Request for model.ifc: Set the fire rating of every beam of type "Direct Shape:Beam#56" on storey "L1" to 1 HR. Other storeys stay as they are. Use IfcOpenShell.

First a look at what the model holds.

```python
import ifcopenshell
import ifcopenshell.util.element

model = ifcopenshell.open("model.ifc")
print(model.schema)
storey = next(s for s in model.by_type("IfcBuildingStorey") if s.Name == "L1")
beams = [e for e in ifcopenshell.util.element.get_decomposition(storey) if e.is_a("IfcBeam")]
seen = {}
for e in beams:
    element_type = ifcopenshell.util.element.get_type(e)
    key = (element_type.Name if element_type != e and element_type else None, ifcopenshell.util.element.get_pset(e, "Pset_BeamCommon", "FireRating"))
    seen[key] = seen.get(key, 0) + 1
for (name, value), count in sorted(seen.items(), key=str):
    print(count, "x", name, "|", value)
```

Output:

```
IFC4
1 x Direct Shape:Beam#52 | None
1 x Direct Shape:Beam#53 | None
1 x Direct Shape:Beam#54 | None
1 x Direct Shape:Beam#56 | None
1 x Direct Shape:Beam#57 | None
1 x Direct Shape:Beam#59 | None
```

```python
import ifcopenshell
import ifcopenshell.api.pset
import ifcopenshell.util.element

model = ifcopenshell.open("model.ifc")

storey = next(s for s in model.by_type("IfcBuildingStorey") if s.Name == "L1")
beams = [e for e in ifcopenshell.util.element.get_decomposition(storey) if e.is_a("IfcBeam")]

count = 0
for e in beams:
    element_type = ifcopenshell.util.element.get_type(e)
    if element_type in (None, e) or element_type.Name != "Direct Shape:Beam#56":
        continue
    # add_pset returns the element's existing set when there is one.
    pset = ifcopenshell.api.pset.add_pset(model, product=e, name="Pset_BeamCommon")
    ifcopenshell.api.pset.edit_pset(model, pset=pset, properties={"FireRating": "1 HR"})
    count += 1

print(count, "beams updated")

model.write("model_updated.ifc")
```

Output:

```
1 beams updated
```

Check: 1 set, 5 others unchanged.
